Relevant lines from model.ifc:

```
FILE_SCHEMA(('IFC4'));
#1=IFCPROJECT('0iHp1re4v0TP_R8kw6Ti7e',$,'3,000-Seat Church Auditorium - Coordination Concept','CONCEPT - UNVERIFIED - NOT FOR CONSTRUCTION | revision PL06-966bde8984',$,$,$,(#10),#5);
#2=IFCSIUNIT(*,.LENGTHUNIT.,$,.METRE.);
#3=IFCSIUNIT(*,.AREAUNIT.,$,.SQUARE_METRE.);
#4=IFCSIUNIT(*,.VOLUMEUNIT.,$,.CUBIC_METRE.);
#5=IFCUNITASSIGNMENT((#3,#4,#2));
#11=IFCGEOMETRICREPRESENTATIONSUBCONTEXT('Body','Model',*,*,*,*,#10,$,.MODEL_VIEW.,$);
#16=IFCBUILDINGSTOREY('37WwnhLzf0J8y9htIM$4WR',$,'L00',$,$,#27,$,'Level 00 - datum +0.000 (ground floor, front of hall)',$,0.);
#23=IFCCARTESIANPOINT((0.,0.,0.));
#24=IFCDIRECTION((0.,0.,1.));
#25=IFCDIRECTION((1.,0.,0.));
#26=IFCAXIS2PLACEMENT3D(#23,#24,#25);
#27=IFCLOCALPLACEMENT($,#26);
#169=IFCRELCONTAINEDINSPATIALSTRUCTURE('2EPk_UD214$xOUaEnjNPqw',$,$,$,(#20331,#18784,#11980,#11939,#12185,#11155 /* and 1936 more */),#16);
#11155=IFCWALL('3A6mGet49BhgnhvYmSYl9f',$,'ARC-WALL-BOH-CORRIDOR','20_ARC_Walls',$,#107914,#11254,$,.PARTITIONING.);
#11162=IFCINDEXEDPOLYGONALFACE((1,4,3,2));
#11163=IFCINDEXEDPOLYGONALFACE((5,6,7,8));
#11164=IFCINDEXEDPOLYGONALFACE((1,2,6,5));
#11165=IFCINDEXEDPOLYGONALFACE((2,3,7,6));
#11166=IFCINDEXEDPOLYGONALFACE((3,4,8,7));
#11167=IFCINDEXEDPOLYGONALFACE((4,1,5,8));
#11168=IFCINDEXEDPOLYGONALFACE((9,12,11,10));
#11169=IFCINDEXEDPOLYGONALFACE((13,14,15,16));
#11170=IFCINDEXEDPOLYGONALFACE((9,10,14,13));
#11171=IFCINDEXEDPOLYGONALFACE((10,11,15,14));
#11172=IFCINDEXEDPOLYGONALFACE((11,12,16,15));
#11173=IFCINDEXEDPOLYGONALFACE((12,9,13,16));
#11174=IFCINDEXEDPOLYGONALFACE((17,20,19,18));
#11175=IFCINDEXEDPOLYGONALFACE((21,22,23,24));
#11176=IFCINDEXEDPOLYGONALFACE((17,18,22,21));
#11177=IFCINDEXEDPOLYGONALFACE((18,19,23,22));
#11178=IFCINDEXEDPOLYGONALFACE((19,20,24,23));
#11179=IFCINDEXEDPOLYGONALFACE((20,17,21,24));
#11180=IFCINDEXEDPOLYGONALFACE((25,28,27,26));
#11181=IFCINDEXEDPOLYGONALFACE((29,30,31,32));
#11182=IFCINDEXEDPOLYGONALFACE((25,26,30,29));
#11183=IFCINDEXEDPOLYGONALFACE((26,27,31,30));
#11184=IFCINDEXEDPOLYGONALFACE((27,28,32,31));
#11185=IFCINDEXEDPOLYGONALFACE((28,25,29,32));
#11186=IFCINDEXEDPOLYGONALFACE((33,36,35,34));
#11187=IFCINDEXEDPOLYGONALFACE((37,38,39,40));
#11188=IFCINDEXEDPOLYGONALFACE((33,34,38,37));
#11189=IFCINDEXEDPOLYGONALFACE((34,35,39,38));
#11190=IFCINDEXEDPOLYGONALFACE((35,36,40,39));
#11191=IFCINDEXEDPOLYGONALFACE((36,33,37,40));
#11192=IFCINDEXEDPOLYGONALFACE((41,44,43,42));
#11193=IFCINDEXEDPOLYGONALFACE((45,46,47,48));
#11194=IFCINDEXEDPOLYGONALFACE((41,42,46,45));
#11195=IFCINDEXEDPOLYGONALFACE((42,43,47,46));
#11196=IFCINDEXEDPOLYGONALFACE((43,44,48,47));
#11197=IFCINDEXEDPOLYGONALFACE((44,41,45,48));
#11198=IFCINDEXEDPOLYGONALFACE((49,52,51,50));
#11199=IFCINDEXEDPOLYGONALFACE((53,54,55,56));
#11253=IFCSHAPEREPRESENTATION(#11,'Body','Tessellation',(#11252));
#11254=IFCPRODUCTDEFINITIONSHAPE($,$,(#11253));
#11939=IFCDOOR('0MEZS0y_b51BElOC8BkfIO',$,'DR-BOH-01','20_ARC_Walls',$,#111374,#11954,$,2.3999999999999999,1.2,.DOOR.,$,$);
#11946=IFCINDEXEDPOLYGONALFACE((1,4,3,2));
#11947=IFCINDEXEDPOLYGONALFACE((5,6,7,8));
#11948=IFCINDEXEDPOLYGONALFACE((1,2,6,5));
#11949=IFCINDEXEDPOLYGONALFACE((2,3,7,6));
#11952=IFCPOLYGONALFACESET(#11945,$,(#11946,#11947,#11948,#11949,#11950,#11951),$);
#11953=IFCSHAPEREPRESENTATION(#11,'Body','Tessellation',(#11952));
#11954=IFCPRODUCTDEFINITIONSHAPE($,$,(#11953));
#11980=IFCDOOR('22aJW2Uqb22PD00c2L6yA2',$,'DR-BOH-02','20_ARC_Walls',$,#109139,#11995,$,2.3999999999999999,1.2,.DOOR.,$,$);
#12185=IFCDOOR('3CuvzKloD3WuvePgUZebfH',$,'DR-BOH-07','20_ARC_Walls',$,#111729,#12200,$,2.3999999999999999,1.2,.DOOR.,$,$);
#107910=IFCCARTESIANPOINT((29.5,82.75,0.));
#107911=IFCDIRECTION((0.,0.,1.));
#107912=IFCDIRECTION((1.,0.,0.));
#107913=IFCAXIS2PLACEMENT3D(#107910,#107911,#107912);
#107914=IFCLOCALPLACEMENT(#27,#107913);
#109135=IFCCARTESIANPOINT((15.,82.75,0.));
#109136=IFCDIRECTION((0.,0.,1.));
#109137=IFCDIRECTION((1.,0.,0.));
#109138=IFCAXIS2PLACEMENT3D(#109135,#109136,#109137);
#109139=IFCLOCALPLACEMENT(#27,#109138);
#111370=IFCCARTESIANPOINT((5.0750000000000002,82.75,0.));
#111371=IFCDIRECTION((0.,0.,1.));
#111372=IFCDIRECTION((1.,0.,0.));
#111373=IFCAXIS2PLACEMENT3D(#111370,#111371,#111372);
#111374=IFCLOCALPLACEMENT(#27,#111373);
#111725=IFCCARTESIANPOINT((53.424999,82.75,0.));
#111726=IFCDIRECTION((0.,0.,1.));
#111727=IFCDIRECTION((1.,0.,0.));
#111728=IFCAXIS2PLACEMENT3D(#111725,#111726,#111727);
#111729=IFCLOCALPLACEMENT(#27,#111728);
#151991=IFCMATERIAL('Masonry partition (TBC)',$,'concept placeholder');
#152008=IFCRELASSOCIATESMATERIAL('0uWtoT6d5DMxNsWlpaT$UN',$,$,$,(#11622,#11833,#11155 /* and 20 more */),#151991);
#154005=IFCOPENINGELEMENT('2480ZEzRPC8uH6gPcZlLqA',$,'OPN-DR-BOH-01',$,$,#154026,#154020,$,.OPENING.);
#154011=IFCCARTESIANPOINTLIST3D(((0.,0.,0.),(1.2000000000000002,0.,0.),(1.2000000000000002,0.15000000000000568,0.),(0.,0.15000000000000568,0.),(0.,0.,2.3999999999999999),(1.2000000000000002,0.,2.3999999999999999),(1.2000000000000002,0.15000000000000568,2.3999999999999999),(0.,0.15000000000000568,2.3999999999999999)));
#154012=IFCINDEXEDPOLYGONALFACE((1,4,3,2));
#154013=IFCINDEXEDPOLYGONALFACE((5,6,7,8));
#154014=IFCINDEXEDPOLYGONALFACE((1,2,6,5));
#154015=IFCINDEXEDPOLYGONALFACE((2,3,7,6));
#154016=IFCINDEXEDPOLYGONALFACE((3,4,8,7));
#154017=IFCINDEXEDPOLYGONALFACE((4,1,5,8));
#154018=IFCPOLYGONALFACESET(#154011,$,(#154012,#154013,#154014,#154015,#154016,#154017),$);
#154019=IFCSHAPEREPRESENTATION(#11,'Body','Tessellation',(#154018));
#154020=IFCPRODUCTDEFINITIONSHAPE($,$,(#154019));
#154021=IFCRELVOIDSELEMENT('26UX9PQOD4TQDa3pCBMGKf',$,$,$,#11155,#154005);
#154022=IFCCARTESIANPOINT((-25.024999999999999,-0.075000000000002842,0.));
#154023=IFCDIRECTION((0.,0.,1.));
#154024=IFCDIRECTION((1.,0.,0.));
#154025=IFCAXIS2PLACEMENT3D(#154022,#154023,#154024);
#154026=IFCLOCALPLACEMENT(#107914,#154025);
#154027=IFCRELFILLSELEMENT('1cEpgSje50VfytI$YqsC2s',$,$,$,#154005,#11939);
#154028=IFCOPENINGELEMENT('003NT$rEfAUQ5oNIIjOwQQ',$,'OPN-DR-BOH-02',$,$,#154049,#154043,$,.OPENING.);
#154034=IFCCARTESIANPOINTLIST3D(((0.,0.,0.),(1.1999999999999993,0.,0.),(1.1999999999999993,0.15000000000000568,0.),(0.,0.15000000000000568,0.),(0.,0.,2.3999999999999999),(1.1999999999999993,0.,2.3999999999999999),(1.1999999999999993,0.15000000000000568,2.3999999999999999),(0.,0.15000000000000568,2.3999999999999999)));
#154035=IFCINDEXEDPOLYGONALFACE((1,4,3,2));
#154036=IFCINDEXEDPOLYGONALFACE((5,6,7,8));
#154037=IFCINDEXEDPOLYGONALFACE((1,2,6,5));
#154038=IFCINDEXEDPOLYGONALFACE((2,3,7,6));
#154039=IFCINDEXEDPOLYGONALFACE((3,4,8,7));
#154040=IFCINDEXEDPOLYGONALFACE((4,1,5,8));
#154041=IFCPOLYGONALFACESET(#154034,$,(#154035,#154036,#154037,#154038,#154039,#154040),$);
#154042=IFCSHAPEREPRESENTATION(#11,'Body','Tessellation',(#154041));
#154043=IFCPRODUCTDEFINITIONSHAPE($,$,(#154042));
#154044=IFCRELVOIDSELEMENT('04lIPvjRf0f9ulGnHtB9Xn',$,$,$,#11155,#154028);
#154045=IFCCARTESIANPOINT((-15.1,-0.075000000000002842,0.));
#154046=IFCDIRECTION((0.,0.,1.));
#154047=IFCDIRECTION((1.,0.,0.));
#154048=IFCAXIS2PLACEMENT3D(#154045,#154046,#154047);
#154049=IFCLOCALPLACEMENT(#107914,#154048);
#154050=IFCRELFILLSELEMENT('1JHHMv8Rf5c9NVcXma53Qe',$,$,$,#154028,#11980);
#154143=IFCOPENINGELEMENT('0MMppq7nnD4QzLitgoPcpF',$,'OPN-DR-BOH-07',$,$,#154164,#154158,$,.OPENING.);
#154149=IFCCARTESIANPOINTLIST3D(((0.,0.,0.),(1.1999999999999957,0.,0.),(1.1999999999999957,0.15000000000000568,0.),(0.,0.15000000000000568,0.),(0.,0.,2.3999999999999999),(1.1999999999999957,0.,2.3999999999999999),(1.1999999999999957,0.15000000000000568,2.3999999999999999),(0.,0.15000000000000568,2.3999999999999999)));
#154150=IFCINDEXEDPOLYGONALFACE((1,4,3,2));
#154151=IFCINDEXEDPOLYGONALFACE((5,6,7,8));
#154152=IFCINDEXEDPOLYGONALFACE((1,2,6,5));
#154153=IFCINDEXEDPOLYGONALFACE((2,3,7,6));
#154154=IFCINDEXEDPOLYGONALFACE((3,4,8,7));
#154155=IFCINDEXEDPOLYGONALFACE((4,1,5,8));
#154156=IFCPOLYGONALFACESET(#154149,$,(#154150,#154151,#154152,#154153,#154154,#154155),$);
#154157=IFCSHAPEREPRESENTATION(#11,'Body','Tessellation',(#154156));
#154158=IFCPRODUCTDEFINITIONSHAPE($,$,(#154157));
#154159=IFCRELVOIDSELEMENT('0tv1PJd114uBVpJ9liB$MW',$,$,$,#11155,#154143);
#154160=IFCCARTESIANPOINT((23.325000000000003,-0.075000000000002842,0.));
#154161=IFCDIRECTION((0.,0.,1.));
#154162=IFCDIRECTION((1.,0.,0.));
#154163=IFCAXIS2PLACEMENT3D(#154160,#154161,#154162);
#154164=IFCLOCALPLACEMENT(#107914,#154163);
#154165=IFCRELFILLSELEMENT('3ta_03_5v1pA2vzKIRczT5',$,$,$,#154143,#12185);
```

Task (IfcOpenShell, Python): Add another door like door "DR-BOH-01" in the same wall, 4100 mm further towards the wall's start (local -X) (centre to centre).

```python
import ifcopenshell
import ifcopenshell.api.feature
import ifcopenshell.api.geometry
import ifcopenshell.api.root
import ifcopenshell.geom
import ifcopenshell.util.element
import ifcopenshell.util.placement
import ifcopenshell.util.shape
import ifcopenshell.util.unit

model = ifcopenshell.open("model.ifc")
unit_scale = ifcopenshell.util.unit.calculate_unit_scale(model)
settings = ifcopenshell.geom.settings()


def volume(element):
    """Net volume in cubic metres, openings subtracted."""
    shape = ifcopenshell.geom.create_shape(settings, element)
    return ifcopenshell.util.shape.get_volume(shape.geometry)


door = model.by_guid("0MEZS0y_b51BElOC8BkfIO")
opening = door.FillsVoids[0].RelatingOpeningElement
wall = opening.VoidsElements[0].RelatingBuildingElement
before = volume(wall)
shift = ifcopenshell.util.placement.get_local_placement(wall.ObjectPlacement)[:3, 0] * -4.1 / unit_scale

# copy_class copies the void relationship, type, container and properties, but no geometry.
new_opening = ifcopenshell.api.root.copy_class(model, product=opening)
new_opening.Representation = ifcopenshell.util.element.copy_deep(
    model, opening.Representation, exclude=["IfcGeometricRepresentationContext", "IfcRepresentationMap"]
)
new_door = ifcopenshell.api.root.copy_class(model, product=door)
new_door.Representation = ifcopenshell.util.element.copy_deep(
    model, door.Representation, exclude=["IfcGeometricRepresentationContext", "IfcRepresentationMap"]
)
ifcopenshell.api.feature.add_filling(model, opening=new_opening, element=new_door)

for old, new in ((opening, new_opening), (door, new_door)):
    matrix = ifcopenshell.util.placement.get_local_placement(old.ObjectPlacement)
    matrix[:3, 3] += shift
    ifcopenshell.api.geometry.edit_object_placement(model, product=new, matrix=matrix, is_si=False)

after = volume(wall)

print(f"wall volume {before:.3f} -> {after:.3f} m3")

model.write("model_updated.ifc")
```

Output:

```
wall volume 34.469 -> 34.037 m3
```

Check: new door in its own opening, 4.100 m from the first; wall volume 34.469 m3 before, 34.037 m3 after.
